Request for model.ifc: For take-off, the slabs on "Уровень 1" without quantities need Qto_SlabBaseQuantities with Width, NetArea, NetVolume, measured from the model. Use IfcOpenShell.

First a look at what the model holds.

```python
import ifcopenshell
import ifcopenshell.util.element
import ifcopenshell.util.unit

model = ifcopenshell.open("model.ifc")
print(model.schema)
for unit_type in ("LENGTHUNIT", "AREAUNIT", "VOLUMEUNIT"):
    print(unit_type, ifcopenshell.util.unit.calculate_unit_scale(model, unit_type))
storey = next(s for s in model.by_type("IfcBuildingStorey") if s.Name == "Уровень 1")
slabs = [e for e in ifcopenshell.util.element.get_decomposition(storey) if e.is_a("IfcSlab")]
for e in sorted(slabs, key=lambda e: e.id()):
    print(e.id(), e.is_a(), e.Name, list(ifcopenshell.util.element.get_psets(e, qtos_only=True)), sep=" | ")
```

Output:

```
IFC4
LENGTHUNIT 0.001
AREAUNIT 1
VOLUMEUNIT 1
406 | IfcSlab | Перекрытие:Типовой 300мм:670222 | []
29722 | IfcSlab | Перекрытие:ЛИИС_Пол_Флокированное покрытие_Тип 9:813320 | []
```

```python
import ifcopenshell
import ifcopenshell.api.pset
import ifcopenshell.geom
import ifcopenshell.util.element
import ifcopenshell.util.shape
import ifcopenshell.util.unit

model = ifcopenshell.open("model.ifc")
unit_scale = ifcopenshell.util.unit.calculate_unit_scale(model)
area_scale = ifcopenshell.util.unit.calculate_unit_scale(model, "AREAUNIT")
volume_scale = ifcopenshell.util.unit.calculate_unit_scale(model, "VOLUMEUNIT")
settings = ifcopenshell.geom.settings()

storey = next(s for s in model.by_type("IfcBuildingStorey") if s.Name == "Уровень 1")
slabs = [e for e in ifcopenshell.util.element.get_decomposition(storey) if e.is_a("IfcSlab")]

for e in sorted(slabs, key=lambda e: e.id()):
    if ifcopenshell.util.element.get_psets(e, qtos_only=True, should_inherit=False):
        continue
    # Geometry comes back in metres, in the element's own axes.
    shape = ifcopenshell.geom.create_shape(settings, e)
    values = {
        "Width": ifcopenshell.util.shape.get_z(shape.geometry) / unit_scale,
        "NetArea": ifcopenshell.util.shape.get_footprint_area(shape.geometry) / area_scale,
        "NetVolume": ifcopenshell.util.shape.get_volume(shape.geometry) / volume_scale,
    }
    qto = ifcopenshell.api.pset.add_qto(model, product=e, name="Qto_SlabBaseQuantities")
    ifcopenshell.api.pset.edit_qto(model, qto=qto, properties=values)
    print(e.id(), {k: round(v, 3) for k, v in values.items()})

model.write("model_edited.ifc")
```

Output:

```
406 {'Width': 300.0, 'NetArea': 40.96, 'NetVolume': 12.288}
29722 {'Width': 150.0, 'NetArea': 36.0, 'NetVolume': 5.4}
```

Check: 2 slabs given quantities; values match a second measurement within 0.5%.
